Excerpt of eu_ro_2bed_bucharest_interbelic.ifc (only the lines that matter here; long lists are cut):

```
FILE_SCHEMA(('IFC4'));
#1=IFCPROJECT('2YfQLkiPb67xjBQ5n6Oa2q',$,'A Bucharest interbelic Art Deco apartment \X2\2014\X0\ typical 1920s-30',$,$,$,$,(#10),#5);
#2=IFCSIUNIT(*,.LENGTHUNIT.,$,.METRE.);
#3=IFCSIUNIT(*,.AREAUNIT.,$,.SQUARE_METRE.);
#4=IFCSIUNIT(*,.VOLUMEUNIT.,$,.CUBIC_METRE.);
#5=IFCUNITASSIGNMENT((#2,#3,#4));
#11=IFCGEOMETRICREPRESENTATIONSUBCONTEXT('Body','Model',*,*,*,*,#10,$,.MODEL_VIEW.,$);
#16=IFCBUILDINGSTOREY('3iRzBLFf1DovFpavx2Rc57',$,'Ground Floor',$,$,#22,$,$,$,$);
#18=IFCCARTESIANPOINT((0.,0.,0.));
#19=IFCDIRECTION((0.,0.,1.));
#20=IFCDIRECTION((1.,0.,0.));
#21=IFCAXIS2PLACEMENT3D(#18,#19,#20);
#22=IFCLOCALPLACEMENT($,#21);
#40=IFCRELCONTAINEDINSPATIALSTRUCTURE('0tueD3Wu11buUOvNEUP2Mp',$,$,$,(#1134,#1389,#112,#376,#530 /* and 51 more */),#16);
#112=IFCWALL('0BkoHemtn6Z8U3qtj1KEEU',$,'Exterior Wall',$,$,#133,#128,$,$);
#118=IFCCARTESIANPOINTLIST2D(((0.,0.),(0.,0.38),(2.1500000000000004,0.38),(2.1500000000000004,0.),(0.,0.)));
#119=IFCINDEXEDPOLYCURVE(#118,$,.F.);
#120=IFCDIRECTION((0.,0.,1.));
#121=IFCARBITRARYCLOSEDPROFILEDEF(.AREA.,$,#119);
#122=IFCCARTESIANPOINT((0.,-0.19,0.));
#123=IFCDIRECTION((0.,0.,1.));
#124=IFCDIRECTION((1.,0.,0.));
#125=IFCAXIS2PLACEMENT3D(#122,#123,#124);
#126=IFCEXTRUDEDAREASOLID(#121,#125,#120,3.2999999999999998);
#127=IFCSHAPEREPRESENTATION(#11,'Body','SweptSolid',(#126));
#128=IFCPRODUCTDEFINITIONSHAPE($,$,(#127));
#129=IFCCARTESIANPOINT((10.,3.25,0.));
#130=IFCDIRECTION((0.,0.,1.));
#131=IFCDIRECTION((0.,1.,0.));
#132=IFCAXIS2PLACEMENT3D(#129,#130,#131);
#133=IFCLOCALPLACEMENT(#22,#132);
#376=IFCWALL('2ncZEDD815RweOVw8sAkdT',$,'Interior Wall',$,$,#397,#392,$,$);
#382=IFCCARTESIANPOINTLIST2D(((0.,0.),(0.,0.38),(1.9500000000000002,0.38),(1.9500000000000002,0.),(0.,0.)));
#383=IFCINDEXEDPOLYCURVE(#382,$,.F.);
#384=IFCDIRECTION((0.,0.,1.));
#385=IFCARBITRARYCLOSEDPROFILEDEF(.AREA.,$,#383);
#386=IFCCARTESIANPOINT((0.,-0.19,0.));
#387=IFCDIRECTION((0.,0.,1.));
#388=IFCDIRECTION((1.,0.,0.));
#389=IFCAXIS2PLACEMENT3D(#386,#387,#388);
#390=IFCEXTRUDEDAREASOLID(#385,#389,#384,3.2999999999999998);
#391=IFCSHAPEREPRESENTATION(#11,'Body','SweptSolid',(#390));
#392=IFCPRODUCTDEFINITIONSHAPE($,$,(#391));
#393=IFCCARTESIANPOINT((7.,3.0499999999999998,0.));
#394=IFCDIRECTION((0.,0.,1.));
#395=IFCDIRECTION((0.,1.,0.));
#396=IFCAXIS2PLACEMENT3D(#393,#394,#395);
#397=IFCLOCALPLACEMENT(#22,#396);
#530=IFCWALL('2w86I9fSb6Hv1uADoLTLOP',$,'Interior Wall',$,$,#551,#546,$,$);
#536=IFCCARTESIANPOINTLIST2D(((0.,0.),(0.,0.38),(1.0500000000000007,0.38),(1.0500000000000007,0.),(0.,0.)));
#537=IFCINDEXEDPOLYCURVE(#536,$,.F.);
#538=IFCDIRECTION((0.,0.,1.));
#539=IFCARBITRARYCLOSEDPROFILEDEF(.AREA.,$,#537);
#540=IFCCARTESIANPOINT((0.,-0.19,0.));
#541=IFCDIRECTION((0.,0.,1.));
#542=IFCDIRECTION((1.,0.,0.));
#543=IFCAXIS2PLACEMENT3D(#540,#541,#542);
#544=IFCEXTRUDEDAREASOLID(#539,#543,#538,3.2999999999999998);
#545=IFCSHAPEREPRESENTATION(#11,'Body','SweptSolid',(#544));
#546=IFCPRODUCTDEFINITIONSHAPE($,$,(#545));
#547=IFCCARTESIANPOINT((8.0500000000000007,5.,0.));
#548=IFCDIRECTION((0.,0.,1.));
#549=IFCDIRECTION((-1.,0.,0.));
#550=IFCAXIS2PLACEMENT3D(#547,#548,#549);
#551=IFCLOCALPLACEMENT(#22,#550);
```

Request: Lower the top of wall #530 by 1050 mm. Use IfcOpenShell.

```python
import ifcopenshell
import ifcopenshell.geom
import ifcopenshell.util.representation
import ifcopenshell.util.shape

model = ifcopenshell.open("eu_ro_2bed_bucharest_interbelic.ifc")
settings = ifcopenshell.geom.settings()


def volume(element):
    """Net volume in cubic metres, openings subtracted."""
    shape = ifcopenshell.geom.create_shape(settings, element)
    return ifcopenshell.util.shape.get_volume(shape.geometry)


wall = model.by_guid("2w86I9fSb6Hv1uADoLTLOP")
before = volume(wall)

body = ifcopenshell.util.representation.get_representation(wall, "Model", "Body")
solid = body.Items[0]
old_height = solid.Depth
solid.Depth -= 1.05
after = volume(wall)

print(f"height {old_height:g} -> {solid.Depth:g}, volume {before:.3f} -> {after:.3f} m3")

model.write("eu_ro_2bed_bucharest_interbelic_edited.ifc")
```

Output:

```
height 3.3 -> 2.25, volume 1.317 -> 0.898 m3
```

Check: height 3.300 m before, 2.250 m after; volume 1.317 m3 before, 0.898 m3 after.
